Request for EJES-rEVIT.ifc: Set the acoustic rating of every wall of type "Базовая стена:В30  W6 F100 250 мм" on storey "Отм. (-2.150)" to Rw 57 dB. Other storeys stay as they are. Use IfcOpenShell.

First a look at what the model holds.

```python
import ifcopenshell
import ifcopenshell.util.element

model = ifcopenshell.open("EJES-rEVIT.ifc")
print(model.schema)
storey = next(s for s in model.by_type("IfcBuildingStorey") if s.Name == "Отм. (-2.150)")
walls = [e for e in ifcopenshell.util.element.get_decomposition(storey) if e.is_a("IfcWall")]
seen = {}
for e in walls:
    element_type = ifcopenshell.util.element.get_type(e)
    key = (element_type.Name if element_type != e and element_type else None, ifcopenshell.util.element.get_pset(e, "Pset_WallCommon", "AcousticRating"))
    seen[key] = seen.get(key, 0) + 1
for (name, value), count in sorted(seen.items(), key=str):
    print(count, "x", name, "|", value)
```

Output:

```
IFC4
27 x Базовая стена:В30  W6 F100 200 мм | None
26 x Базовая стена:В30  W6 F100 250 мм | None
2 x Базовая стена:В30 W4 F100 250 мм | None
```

```python
import ifcopenshell
import ifcopenshell.api.pset
import ifcopenshell.util.element

model = ifcopenshell.open("EJES-rEVIT.ifc")

storey = next(s for s in model.by_type("IfcBuildingStorey") if s.Name == "Отм. (-2.150)")
walls = [e for e in ifcopenshell.util.element.get_decomposition(storey) if e.is_a("IfcWall")]

count = 0
for e in walls:
    element_type = ifcopenshell.util.element.get_type(e)
    if element_type in (None, e) or element_type.Name != "Базовая стена:В30  W6 F100 250 мм":
        continue
    # add_pset returns the element's existing set when there is one.
    pset = ifcopenshell.api.pset.add_pset(model, product=e, name="Pset_WallCommon")
    ifcopenshell.api.pset.edit_pset(model, pset=pset, properties={"AcousticRating": "Rw 57 dB"})
    count += 1

print(count, "walls updated")

model.write("EJES-rEVIT_rev.ifc")
```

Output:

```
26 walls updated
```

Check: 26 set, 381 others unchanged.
